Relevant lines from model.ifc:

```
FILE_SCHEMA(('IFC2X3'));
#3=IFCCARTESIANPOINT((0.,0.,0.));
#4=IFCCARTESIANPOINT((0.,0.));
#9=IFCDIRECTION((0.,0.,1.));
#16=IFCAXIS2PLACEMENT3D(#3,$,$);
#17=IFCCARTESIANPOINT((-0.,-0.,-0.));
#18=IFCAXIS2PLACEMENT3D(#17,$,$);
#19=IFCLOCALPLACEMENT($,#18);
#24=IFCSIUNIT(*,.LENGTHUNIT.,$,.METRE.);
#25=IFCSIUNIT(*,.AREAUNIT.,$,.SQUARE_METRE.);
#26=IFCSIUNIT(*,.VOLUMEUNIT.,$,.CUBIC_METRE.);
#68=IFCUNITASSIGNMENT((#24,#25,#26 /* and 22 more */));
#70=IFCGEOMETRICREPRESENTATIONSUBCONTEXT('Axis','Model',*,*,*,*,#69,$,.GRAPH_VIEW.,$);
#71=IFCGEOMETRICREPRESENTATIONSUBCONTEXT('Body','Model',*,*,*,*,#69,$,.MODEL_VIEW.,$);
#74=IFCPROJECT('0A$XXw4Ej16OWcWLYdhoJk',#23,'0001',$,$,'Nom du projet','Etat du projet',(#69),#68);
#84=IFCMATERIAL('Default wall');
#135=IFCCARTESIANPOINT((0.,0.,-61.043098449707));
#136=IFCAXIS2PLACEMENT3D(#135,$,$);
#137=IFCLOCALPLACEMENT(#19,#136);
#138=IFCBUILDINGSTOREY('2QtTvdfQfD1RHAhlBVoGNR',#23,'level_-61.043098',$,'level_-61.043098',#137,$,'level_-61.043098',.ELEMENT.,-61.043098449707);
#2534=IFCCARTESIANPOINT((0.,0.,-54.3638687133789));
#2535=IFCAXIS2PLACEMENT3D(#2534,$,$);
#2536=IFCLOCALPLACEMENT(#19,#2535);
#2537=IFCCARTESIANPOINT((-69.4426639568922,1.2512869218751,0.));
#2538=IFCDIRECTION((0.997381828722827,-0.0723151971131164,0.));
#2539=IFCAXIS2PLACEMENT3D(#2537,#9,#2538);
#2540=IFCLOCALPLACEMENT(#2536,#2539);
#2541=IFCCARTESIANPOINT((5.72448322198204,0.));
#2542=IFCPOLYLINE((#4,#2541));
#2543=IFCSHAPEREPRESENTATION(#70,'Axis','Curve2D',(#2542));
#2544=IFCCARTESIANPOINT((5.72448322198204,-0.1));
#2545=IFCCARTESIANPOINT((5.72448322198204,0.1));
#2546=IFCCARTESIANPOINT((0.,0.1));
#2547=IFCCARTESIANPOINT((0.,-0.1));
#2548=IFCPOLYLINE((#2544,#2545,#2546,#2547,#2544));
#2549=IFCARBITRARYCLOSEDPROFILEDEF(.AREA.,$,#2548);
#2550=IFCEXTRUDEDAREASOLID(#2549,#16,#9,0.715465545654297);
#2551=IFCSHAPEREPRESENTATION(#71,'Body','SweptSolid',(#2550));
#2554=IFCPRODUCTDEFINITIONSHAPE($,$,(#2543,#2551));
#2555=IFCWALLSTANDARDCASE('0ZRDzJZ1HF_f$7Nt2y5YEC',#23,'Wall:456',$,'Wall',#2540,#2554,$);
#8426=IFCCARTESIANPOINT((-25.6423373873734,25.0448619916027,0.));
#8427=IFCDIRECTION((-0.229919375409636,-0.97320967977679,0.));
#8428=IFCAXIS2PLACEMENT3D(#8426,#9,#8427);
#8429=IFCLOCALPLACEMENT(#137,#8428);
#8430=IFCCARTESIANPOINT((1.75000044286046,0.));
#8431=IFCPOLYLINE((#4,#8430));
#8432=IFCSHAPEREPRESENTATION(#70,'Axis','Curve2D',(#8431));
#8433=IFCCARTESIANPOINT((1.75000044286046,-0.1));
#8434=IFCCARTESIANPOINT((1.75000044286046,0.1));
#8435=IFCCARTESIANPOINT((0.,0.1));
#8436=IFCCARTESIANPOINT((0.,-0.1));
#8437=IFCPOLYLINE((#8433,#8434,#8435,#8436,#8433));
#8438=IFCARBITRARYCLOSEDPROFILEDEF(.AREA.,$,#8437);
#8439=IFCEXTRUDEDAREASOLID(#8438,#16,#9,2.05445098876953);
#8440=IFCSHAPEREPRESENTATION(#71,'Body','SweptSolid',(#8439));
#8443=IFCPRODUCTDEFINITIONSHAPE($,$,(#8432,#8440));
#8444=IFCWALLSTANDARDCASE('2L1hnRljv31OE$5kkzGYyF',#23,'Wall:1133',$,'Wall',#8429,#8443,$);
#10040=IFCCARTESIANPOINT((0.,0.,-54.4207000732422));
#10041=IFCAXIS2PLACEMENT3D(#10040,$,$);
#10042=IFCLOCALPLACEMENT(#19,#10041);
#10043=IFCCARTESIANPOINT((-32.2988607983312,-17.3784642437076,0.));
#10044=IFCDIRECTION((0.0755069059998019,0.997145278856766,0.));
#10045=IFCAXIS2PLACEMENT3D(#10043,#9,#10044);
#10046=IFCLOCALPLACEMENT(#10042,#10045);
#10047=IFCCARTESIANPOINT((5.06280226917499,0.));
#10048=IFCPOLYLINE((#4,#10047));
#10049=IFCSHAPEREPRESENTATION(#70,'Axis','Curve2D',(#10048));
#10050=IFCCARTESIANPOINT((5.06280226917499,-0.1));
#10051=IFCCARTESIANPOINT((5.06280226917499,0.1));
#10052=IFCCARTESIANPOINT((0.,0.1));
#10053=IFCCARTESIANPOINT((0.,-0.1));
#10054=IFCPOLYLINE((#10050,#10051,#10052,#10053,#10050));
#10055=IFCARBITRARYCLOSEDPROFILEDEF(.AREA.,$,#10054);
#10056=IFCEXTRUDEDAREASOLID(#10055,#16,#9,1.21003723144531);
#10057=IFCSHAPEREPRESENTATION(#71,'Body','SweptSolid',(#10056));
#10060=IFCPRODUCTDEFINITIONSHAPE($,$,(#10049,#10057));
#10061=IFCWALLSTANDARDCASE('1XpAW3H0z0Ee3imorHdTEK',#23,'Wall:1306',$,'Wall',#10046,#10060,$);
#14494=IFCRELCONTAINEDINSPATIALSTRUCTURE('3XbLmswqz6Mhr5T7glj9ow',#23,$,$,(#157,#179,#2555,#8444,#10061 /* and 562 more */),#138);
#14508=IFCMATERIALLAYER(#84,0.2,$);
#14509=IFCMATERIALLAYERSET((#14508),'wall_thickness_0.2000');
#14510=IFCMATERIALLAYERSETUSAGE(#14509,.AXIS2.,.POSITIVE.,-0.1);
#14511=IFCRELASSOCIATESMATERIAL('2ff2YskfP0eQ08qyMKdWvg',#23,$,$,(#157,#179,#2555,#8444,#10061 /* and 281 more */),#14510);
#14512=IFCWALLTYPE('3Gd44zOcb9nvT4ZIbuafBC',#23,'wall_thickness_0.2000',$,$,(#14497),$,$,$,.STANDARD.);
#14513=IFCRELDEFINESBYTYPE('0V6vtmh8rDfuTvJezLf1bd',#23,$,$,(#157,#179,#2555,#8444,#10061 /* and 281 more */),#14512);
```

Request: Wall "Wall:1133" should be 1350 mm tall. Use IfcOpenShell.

```python
import ifcopenshell
import ifcopenshell.geom
import ifcopenshell.util.representation
import ifcopenshell.util.shape
import ifcopenshell.util.unit

model = ifcopenshell.open("model.ifc")
unit_scale = ifcopenshell.util.unit.calculate_unit_scale(model)
settings = ifcopenshell.geom.settings()


def volume(element):
    """Net volume in cubic metres, openings subtracted."""
    shape = ifcopenshell.geom.create_shape(settings, element)
    return ifcopenshell.util.shape.get_volume(shape.geometry)


wall = model.by_guid("2L1hnRljv31OE$5kkzGYyF")
before = volume(wall)

body = ifcopenshell.util.representation.get_representation(wall, "Model", "Body")
solid = body.Items[0]
old_height = solid.Depth
solid.Depth = 1.35 / unit_scale
after = volume(wall)

print(f"height {old_height:g} -> {solid.Depth:g}, volume {before:.3f} -> {after:.3f} m3")

model.write("model_updated.ifc")
```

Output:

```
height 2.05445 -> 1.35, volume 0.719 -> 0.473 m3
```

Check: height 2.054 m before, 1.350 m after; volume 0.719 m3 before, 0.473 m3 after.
